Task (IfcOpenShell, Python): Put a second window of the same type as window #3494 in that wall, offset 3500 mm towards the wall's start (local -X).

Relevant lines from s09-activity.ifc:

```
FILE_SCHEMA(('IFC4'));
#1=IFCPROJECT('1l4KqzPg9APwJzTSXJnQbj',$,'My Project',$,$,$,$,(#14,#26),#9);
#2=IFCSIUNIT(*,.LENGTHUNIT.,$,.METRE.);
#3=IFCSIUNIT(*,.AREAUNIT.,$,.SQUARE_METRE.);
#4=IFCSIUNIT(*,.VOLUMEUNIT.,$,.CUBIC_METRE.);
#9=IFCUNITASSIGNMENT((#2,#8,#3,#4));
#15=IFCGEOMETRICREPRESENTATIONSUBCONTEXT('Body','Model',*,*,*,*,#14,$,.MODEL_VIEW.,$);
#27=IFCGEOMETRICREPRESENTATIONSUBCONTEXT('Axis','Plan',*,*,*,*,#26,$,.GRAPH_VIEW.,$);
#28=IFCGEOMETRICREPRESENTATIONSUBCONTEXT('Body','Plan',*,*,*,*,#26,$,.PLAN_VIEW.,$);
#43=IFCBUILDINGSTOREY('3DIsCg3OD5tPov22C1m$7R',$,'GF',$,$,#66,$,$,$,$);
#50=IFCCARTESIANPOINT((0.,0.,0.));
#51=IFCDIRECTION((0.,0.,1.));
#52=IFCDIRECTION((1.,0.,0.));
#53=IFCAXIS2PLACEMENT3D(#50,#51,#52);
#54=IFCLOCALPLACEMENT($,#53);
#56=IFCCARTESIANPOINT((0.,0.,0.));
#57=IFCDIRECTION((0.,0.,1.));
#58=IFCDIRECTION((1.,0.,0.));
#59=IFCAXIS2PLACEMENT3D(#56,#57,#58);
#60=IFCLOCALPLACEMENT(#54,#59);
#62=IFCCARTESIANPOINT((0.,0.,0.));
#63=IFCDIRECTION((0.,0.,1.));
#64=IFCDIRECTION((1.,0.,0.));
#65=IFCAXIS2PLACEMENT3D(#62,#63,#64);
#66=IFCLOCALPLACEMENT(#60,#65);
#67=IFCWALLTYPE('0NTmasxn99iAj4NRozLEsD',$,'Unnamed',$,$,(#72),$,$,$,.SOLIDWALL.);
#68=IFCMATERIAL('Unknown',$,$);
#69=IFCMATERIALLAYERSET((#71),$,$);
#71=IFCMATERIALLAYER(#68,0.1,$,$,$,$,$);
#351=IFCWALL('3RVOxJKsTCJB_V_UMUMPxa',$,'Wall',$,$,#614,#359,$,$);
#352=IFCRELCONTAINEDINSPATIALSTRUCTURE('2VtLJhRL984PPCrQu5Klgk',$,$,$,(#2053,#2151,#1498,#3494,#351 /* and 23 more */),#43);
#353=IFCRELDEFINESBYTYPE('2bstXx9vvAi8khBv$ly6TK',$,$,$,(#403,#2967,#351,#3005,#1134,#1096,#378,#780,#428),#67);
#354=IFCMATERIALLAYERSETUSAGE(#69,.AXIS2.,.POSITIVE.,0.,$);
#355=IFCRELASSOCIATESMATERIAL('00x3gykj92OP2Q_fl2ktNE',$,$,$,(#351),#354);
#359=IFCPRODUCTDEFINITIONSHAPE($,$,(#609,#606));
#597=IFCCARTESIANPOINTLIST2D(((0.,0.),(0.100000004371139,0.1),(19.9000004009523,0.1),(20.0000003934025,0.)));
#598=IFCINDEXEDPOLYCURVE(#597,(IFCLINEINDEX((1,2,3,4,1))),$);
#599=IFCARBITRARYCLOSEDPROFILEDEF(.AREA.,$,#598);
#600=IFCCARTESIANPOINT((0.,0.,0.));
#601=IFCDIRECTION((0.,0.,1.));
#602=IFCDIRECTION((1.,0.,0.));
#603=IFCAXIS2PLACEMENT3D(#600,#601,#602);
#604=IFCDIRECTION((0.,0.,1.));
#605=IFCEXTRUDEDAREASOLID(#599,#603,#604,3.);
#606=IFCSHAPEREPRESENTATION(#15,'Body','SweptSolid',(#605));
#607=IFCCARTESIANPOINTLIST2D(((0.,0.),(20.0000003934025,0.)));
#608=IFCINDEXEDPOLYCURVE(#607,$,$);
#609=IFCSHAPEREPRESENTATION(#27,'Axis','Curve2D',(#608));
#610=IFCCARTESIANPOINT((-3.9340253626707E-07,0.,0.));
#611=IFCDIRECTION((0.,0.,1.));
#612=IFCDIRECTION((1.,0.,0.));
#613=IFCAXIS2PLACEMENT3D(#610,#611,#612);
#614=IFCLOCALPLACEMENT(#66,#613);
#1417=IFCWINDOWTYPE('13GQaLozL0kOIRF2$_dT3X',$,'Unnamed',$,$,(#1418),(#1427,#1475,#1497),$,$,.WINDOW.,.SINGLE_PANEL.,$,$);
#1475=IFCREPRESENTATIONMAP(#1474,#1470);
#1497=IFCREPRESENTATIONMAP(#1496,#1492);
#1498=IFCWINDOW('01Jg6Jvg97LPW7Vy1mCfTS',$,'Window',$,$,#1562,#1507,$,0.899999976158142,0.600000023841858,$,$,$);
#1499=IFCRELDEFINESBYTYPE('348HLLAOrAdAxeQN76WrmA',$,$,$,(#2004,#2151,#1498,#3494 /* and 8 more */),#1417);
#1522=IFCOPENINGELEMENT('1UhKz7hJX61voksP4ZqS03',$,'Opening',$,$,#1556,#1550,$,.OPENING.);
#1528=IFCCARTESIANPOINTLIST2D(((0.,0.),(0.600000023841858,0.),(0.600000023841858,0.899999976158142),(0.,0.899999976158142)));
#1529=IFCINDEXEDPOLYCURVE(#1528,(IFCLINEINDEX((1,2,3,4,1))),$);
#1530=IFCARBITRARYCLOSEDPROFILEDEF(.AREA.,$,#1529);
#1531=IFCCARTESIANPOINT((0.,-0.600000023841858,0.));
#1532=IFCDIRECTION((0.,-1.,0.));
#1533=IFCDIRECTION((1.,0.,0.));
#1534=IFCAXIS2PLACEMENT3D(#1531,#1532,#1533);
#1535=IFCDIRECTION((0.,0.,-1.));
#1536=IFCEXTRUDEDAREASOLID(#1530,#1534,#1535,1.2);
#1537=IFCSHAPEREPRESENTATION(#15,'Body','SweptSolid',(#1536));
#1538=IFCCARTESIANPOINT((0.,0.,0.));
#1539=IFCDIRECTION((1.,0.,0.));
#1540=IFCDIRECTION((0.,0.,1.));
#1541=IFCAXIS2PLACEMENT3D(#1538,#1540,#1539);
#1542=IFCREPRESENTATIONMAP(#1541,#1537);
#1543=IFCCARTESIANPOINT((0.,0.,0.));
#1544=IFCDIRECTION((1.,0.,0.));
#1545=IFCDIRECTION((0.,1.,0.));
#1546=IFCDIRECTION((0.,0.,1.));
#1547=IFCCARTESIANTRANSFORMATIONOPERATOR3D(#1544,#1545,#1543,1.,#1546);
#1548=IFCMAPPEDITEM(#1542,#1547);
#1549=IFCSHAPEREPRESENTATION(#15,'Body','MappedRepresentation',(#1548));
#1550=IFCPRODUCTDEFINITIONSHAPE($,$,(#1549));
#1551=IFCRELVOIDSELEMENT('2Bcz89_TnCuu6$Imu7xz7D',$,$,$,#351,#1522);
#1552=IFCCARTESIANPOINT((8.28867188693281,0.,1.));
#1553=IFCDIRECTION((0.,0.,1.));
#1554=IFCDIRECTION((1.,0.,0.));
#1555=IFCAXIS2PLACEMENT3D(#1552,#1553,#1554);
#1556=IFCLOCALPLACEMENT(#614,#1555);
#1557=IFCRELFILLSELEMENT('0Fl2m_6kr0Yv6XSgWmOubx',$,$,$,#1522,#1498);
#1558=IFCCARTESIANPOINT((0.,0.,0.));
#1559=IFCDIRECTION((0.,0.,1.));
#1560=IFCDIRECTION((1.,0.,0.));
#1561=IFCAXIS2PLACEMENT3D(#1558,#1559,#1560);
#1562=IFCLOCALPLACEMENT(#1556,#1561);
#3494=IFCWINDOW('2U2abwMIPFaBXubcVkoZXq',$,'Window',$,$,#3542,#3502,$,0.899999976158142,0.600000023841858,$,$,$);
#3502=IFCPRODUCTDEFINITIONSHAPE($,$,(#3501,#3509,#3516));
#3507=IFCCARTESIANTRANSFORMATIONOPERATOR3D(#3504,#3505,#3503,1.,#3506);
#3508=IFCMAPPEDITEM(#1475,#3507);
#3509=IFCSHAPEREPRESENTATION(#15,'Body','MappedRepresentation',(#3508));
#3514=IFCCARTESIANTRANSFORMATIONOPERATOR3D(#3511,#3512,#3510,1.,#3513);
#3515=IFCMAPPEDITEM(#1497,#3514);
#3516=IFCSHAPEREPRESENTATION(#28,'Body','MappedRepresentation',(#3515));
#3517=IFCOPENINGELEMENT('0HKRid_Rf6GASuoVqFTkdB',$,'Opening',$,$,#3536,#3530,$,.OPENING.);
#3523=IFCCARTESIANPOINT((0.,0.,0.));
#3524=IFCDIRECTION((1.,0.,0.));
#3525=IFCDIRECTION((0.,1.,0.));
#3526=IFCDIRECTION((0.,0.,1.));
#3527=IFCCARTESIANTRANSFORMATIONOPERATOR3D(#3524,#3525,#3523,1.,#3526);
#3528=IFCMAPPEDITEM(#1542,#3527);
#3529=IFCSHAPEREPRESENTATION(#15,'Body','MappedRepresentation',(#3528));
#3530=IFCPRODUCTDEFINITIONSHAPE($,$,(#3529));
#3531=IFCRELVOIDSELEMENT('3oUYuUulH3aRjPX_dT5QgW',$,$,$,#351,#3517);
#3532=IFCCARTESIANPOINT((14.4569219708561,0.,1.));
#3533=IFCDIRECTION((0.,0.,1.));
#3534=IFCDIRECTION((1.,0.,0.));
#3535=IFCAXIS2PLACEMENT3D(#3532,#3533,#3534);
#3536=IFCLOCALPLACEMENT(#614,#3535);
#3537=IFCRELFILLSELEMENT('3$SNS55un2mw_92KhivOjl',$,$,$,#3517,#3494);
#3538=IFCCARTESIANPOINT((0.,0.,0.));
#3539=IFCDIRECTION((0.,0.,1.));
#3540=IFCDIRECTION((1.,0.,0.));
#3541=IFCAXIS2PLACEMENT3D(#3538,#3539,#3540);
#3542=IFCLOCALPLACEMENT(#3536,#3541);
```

```python
import ifcopenshell
import ifcopenshell.api.feature
import ifcopenshell.api.geometry
import ifcopenshell.api.root
import ifcopenshell.geom
import ifcopenshell.util.element
import ifcopenshell.util.placement
import ifcopenshell.util.shape

model = ifcopenshell.open("s09-activity.ifc")
settings = ifcopenshell.geom.settings()


def volume(element):
    """Net volume in cubic metres, openings subtracted."""
    shape = ifcopenshell.geom.create_shape(settings, element)
    return ifcopenshell.util.shape.get_volume(shape.geometry)


window = model.by_id(3494)
opening = window.FillsVoids[0].RelatingOpeningElement
wall = opening.VoidsElements[0].RelatingBuildingElement
before = volume(wall)
shift = ifcopenshell.util.placement.get_local_placement(wall.ObjectPlacement)[:3, 0] * -3.5

# copy_class copies the void relationship, type, container and properties, but no geometry.
new_opening = ifcopenshell.api.root.copy_class(model, product=opening)
new_opening.Representation = ifcopenshell.util.element.copy_deep(
    model, opening.Representation, exclude=["IfcGeometricRepresentationContext", "IfcRepresentationMap"]
)
new_window = ifcopenshell.api.root.copy_class(model, product=window)
new_window.Representation = ifcopenshell.util.element.copy_deep(
    model, window.Representation, exclude=["IfcGeometricRepresentationContext", "IfcRepresentationMap"]
)
ifcopenshell.api.feature.add_filling(model, opening=new_opening, element=new_window)

for old, new in ((opening, new_opening), (window, new_window)):
    matrix = ifcopenshell.util.placement.get_local_placement(old.ObjectPlacement)
    matrix[:3, 3] += shift
    ifcopenshell.api.geometry.edit_object_placement(model, product=new, matrix=matrix, is_si=False)

after = volume(wall)

print(f"wall volume {before:.3f} -> {after:.3f} m3")

model.write("s09-activity-out.ifc")
```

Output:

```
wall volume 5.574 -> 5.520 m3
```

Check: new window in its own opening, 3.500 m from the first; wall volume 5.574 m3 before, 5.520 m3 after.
